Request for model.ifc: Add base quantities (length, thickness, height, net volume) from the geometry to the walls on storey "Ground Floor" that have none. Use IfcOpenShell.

First a look at what the model holds.

```python
import ifcopenshell
import ifcopenshell.util.element
import ifcopenshell.util.unit

model = ifcopenshell.open("model.ifc")
print(model.schema)
for unit_type in ("LENGTHUNIT", "AREAUNIT", "VOLUMEUNIT"):
    print(unit_type, ifcopenshell.util.unit.calculate_unit_scale(model, unit_type))
storey = next(s for s in model.by_type("IfcBuildingStorey") if s.Name == "Ground Floor")
walls = [e for e in ifcopenshell.util.element.get_decomposition(storey) if e.is_a("IfcWall")]
for e in sorted(walls, key=lambda e: e.id()):
    print(e.id(), e.is_a(), e.Name, list(ifcopenshell.util.element.get_psets(e, qtos_only=True)), sep=" | ")
```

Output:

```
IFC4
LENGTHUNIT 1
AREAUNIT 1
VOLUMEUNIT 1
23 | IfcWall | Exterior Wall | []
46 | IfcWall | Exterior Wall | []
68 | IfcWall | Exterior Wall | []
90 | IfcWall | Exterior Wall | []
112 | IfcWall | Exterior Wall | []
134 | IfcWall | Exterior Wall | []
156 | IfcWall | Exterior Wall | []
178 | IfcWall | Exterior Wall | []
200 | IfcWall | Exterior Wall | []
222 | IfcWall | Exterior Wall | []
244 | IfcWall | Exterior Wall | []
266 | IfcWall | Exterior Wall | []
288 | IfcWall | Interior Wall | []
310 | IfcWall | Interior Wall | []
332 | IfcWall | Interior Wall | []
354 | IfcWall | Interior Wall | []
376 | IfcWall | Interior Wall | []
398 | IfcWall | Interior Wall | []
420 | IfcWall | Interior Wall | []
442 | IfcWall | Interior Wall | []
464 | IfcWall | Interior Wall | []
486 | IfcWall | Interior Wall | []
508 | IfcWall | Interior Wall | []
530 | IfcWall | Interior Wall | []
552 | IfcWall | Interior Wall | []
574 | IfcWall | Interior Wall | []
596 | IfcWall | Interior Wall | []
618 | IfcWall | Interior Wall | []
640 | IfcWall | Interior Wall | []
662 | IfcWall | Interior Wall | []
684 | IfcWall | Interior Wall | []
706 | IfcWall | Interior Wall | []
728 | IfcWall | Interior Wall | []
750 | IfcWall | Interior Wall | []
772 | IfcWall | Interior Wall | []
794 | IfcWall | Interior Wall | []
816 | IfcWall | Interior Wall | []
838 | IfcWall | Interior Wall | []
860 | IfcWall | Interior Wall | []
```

```python
import ifcopenshell
import ifcopenshell.api.pset
import ifcopenshell.geom
import ifcopenshell.util.element
import ifcopenshell.util.shape
import ifcopenshell.util.unit

model = ifcopenshell.open("model.ifc")
unit_scale = ifcopenshell.util.unit.calculate_unit_scale(model)
volume_scale = ifcopenshell.util.unit.calculate_unit_scale(model, "VOLUMEUNIT")
settings = ifcopenshell.geom.settings()

storey = next(s for s in model.by_type("IfcBuildingStorey") if s.Name == "Ground Floor")
walls = [e for e in ifcopenshell.util.element.get_decomposition(storey) if e.is_a("IfcWall")]

for e in sorted(walls, key=lambda e: e.id()):
    if ifcopenshell.util.element.get_psets(e, qtos_only=True, should_inherit=False):
        continue
    # Geometry comes back in metres, in the element's own axes.
    shape = ifcopenshell.geom.create_shape(settings, e)
    values = {
        "Length": ifcopenshell.util.shape.get_x(shape.geometry) / unit_scale,
        "Width": ifcopenshell.util.shape.get_y(shape.geometry) / unit_scale,
        "Height": ifcopenshell.util.shape.get_z(shape.geometry) / unit_scale,
        "NetVolume": ifcopenshell.util.shape.get_volume(shape.geometry) / volume_scale,
    }
    qto = ifcopenshell.api.pset.add_qto(model, product=e, name="Qto_WallBaseQuantities")
    ifcopenshell.api.pset.edit_qto(model, qto=qto, properties=values)
    print(e.id(), {k: round(v, 3) for k, v in values.items()})

model.write("model_edited.ifc")
```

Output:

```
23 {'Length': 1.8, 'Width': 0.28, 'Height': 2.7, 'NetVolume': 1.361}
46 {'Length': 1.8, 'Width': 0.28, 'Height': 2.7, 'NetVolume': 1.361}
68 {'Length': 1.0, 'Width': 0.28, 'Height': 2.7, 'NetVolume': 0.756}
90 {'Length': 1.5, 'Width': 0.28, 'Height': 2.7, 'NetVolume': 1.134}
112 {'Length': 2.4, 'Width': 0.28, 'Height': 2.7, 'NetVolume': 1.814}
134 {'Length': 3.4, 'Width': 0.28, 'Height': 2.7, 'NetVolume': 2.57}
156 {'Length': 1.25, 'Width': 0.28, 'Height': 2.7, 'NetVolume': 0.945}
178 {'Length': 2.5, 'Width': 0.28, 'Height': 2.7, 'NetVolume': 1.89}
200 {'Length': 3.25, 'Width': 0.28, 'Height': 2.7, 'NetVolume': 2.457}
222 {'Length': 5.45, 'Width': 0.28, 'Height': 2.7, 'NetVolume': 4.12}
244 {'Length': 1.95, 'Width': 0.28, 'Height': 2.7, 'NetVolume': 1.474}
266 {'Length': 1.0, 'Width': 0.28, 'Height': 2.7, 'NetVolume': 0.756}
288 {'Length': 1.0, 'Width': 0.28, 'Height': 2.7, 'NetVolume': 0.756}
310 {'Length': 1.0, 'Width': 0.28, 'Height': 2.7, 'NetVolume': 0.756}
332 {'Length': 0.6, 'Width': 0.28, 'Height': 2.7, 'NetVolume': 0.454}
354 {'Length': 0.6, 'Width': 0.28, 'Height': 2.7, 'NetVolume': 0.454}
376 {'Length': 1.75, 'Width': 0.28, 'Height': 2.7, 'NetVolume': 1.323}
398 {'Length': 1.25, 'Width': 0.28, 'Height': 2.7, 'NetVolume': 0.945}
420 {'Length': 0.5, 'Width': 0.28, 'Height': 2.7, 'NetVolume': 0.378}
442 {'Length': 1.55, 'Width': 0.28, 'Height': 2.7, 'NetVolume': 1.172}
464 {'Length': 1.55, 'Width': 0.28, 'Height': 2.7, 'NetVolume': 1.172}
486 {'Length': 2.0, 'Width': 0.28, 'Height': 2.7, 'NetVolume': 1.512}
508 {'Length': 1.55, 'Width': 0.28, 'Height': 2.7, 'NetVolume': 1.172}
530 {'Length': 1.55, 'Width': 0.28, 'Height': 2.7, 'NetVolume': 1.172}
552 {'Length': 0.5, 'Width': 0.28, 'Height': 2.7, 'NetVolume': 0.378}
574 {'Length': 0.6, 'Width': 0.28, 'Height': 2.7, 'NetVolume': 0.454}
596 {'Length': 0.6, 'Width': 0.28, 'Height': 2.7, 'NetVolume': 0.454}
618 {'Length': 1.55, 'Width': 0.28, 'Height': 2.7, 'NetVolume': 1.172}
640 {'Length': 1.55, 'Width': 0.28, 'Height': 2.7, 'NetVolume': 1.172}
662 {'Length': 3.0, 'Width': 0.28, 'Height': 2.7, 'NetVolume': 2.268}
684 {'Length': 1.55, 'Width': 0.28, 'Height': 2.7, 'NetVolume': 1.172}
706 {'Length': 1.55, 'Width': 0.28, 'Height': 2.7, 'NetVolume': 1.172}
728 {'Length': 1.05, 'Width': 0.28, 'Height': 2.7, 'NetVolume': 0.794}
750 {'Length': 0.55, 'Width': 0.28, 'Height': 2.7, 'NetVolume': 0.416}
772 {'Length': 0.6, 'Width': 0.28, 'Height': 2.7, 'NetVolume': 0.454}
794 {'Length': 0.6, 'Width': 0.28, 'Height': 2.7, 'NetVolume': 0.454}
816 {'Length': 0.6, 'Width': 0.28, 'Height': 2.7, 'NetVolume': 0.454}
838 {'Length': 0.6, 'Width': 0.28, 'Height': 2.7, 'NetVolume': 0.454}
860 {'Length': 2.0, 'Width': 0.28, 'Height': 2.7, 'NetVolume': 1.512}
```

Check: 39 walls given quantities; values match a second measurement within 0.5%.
